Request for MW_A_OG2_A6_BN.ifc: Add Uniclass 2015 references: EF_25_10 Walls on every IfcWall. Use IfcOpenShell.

First a look at what the model holds.

```python
import ifcopenshell

model = ifcopenshell.open("MW_A_OG2_A6_BN.ifc")
print(model.schema)
print("classifications:", [c.Name for c in model.by_type("IfcClassification")])
for ifc_class in ("IfcDoor", "IfcRoof", "IfcStair", "IfcWall", "IfcWindow"):
    print(ifc_class, len(model.by_type(ifc_class)))
```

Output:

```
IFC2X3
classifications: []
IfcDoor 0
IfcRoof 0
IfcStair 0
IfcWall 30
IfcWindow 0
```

```python
import ifcopenshell
import ifcopenshell.api.classification

model = ifcopenshell.open("MW_A_OG2_A6_BN.ifc")

# IFC2X3 requires Source and Edition and has no link from the project to the system.
system = model.create_entity("IfcClassification", Source="NBS", Edition="2015", Name="Uniclass 2015")

codes = {
    "IfcWall": ("EF_25_10", "Walls"),
}
for ifc_class, (code, name) in codes.items():
    products = model.by_type(ifc_class)
    ifcopenshell.api.classification.add_reference(
        model, products=products, classification=system, identification=code, name=name
    )
    print(code, len(products))

model.write("MW_A_OG2_A6_BN_v2.ifc")
```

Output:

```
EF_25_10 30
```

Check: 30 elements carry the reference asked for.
